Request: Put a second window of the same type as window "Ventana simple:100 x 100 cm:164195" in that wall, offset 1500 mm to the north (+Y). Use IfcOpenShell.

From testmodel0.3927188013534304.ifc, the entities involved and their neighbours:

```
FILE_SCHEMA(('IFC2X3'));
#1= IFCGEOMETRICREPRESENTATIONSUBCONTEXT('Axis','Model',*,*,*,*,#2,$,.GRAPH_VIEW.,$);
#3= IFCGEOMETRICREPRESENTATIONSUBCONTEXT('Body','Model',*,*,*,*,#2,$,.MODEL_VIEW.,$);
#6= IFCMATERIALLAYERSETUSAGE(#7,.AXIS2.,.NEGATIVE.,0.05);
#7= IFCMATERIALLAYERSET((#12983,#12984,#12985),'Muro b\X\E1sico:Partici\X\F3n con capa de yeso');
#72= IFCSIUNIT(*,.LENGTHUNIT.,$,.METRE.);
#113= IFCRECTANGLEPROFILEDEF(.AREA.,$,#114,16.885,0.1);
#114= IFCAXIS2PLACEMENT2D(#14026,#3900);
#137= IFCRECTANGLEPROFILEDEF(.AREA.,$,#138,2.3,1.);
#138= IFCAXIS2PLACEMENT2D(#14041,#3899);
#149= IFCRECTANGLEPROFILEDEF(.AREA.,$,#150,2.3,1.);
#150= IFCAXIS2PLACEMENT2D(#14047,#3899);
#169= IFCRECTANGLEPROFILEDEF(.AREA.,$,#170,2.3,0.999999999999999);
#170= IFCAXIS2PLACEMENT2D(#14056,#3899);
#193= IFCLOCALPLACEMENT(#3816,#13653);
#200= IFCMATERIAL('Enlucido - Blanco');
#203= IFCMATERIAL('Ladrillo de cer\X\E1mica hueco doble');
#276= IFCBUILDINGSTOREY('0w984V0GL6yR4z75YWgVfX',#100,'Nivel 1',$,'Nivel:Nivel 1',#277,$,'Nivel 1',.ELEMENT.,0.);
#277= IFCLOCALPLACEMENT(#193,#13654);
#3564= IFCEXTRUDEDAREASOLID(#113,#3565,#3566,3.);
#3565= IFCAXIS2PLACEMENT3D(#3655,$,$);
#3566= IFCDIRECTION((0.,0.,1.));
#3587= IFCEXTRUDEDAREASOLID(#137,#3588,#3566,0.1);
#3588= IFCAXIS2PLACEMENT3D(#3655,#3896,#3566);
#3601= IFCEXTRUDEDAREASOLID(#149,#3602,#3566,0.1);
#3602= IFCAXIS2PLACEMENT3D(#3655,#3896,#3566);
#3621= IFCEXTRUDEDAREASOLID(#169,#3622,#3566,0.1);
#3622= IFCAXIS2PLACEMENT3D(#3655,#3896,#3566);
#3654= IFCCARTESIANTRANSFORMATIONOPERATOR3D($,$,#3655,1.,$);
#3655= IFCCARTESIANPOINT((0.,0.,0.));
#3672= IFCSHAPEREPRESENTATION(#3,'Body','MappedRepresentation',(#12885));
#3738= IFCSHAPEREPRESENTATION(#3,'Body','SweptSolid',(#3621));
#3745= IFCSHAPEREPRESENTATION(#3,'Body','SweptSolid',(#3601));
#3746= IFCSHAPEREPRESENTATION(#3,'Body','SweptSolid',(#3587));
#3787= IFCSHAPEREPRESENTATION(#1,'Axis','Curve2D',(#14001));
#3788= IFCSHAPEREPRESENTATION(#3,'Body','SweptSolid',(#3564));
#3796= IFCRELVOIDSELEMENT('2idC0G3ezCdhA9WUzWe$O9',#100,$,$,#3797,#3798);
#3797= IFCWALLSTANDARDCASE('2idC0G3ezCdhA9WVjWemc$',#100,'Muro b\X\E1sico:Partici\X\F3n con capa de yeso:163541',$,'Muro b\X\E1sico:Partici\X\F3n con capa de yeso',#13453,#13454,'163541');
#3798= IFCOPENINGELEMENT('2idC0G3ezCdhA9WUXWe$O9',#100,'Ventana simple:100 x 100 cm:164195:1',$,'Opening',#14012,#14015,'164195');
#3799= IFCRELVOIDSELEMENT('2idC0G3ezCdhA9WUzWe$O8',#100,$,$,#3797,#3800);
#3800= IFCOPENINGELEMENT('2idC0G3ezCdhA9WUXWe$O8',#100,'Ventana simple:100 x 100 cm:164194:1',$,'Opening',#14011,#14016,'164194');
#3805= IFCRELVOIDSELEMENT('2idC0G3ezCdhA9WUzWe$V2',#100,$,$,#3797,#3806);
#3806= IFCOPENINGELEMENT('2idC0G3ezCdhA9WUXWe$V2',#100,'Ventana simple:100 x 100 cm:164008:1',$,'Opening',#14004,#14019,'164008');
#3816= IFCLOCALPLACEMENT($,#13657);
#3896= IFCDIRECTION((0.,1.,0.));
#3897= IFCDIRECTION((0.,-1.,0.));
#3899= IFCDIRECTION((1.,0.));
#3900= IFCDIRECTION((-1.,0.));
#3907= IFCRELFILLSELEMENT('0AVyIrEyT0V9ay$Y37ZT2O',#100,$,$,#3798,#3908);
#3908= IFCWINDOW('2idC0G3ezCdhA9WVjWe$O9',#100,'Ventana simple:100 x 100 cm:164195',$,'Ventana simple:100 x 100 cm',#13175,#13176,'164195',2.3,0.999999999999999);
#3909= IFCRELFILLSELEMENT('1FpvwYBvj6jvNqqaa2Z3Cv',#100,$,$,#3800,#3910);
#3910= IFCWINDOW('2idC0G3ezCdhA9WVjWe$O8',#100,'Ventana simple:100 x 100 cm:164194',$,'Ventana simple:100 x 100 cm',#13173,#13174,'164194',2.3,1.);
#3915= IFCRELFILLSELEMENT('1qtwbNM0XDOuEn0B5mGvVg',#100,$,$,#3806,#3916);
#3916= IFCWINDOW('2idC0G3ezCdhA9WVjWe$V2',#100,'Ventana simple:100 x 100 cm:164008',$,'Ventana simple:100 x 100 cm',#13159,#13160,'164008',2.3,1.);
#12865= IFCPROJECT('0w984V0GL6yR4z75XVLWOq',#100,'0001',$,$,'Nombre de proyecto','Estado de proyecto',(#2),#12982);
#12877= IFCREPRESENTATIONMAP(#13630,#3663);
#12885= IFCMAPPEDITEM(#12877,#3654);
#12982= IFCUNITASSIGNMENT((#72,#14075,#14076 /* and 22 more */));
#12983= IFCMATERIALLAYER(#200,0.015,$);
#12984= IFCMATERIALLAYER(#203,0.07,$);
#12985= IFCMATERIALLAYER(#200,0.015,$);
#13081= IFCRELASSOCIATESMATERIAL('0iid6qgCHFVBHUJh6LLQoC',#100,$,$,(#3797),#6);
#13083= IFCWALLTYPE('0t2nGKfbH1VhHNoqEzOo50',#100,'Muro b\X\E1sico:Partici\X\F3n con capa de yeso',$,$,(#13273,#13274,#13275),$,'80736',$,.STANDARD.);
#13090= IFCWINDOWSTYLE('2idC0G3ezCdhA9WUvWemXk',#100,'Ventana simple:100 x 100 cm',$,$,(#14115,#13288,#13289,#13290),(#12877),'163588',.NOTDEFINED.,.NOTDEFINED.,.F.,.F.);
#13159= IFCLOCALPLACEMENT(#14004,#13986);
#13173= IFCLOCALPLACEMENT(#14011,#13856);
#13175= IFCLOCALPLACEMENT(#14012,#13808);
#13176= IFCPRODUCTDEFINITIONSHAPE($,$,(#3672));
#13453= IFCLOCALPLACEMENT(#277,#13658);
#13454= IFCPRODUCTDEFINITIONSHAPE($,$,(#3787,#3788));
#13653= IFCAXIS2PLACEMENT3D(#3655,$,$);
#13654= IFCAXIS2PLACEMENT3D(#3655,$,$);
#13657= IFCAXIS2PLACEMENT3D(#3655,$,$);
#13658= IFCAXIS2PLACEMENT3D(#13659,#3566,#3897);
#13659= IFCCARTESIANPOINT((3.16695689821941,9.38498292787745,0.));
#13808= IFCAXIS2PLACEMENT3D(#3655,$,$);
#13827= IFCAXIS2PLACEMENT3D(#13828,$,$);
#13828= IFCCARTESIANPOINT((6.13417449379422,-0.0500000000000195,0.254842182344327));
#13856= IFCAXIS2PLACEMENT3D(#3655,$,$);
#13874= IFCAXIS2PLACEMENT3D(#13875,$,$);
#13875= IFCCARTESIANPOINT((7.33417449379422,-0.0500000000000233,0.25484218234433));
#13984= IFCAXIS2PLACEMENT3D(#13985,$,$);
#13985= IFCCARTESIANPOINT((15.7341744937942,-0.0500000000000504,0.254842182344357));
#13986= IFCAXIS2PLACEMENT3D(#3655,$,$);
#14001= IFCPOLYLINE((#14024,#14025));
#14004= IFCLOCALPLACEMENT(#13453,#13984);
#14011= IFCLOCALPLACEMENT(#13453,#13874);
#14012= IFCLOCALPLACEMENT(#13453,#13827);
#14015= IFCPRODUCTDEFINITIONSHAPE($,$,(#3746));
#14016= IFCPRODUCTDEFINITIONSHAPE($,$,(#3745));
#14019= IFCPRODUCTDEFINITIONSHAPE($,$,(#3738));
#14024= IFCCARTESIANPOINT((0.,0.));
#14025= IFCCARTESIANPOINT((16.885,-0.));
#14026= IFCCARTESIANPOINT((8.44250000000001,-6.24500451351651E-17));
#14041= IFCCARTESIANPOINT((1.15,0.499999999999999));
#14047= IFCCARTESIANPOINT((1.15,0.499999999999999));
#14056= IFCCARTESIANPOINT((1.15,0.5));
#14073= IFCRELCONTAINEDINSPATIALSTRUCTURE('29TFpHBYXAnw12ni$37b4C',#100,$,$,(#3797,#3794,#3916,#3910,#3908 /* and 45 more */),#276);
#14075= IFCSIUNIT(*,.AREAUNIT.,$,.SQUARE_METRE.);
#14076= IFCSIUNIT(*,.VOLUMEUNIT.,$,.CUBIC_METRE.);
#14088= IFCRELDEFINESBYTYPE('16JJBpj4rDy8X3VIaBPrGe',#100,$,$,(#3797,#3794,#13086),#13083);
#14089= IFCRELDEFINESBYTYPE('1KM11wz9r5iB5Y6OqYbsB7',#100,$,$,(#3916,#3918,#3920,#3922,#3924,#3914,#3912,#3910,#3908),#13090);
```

```python
import ifcopenshell
import ifcopenshell.api.feature
import ifcopenshell.api.geometry
import ifcopenshell.api.root
import ifcopenshell.geom
import ifcopenshell.util.element
import ifcopenshell.util.placement
import ifcopenshell.util.shape

model = ifcopenshell.open("testmodel0.3927188013534304.ifc")
settings = ifcopenshell.geom.settings()


def volume(element):
    """Net volume in cubic metres, openings subtracted."""
    shape = ifcopenshell.geom.create_shape(settings, element)
    return ifcopenshell.util.shape.get_volume(shape.geometry)


def reuse_history(source, copy):
    """copy_class also copies each property set's owner history, people and application; keep the originals."""
    for rel in copy.IsDefinedBy:
        if rel.is_a("IfcRelDefinesByProperties") and (history := rel.RelatingPropertyDefinition.OwnerHistory):
            rel.RelatingPropertyDefinition.OwnerHistory = source.OwnerHistory
            ifcopenshell.util.element.remove_deep2(model, history)


window = model.by_id(3908)
opening = window.FillsVoids[0].RelatingOpeningElement
wall = opening.VoidsElements[0].RelatingBuildingElement
before = volume(wall)
shift = ifcopenshell.util.placement.get_local_placement(wall.ObjectPlacement)[:3, 0] * -1.5

# copy_class copies the void relationship, type, container and properties, but no geometry.
new_opening = ifcopenshell.api.root.copy_class(model, product=opening)
new_opening.Representation = ifcopenshell.util.element.copy_deep(
    model, opening.Representation, exclude=["IfcGeometricRepresentationContext", "IfcRepresentationMap"]
)
new_opening.Name = "Ventana simple:100 x 100 cm"
new_opening.Tag = None
new_window = ifcopenshell.api.root.copy_class(model, product=window)
new_window.Representation = ifcopenshell.util.element.copy_deep(
    model, window.Representation, exclude=["IfcGeometricRepresentationContext", "IfcRepresentationMap"]
)
new_window.Name = "Ventana simple:100 x 100 cm"
new_window.Tag = None
reuse_history(window, new_window)
fills = ifcopenshell.api.feature.add_filling(model, opening=new_opening, element=new_window)
fills.OwnerHistory = new_window.OwnerHistory  # required in IFC2X3

for old, new in ((opening, new_opening), (window, new_window)):
    matrix = ifcopenshell.util.placement.get_local_placement(old.ObjectPlacement)
    matrix[:3, 3] += shift
    ifcopenshell.api.geometry.edit_object_placement(model, product=new, matrix=matrix, is_si=False)

after = volume(wall)

print(f"wall volume {before:.3f} -> {after:.3f} m3")

model.write("testmodel0.3927188013534304_updated.ifc")
```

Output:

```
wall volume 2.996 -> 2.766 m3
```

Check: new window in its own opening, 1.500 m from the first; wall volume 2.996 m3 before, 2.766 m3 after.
